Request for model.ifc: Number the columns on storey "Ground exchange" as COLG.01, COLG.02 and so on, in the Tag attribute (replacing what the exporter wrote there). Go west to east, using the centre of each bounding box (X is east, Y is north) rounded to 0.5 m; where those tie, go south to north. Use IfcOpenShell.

First a look at what the model holds.

```python
import ifcopenshell
import ifcopenshell.util.element
import ifcopenshell.util.placement

model = ifcopenshell.open("model.ifc")
print(model.schema)
storey = next(s for s in model.by_type("IfcBuildingStorey") if s.Name == "Ground exchange")
columns = [e for e in ifcopenshell.util.element.get_decomposition(storey) if e.is_a("IfcColumn")]
for e in sorted(columns, key=lambda e: e.id()):
    origin = ifcopenshell.util.placement.get_local_placement(e.ObjectPlacement)[:3, 3]
    print(e.id(), e.Tag, e.Name, origin.round(2) + 0.0, sep=" | ")
```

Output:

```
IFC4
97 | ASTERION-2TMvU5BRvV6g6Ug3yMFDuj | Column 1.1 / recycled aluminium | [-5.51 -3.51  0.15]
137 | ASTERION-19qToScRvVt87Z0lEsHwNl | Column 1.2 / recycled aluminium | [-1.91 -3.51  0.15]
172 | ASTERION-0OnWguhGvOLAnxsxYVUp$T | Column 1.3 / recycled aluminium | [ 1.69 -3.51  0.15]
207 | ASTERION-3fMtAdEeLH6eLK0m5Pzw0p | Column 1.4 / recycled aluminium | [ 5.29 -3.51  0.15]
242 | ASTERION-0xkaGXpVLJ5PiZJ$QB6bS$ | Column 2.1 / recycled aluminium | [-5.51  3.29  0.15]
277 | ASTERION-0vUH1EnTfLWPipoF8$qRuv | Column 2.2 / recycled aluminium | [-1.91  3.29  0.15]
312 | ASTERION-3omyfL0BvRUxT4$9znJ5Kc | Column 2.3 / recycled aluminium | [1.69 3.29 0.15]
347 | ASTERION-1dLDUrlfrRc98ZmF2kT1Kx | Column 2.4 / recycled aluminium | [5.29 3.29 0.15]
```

```python
import ifcopenshell
import ifcopenshell.geom
import ifcopenshell.util.element
import ifcopenshell.util.shape

model = ifcopenshell.open("model.ifc")
settings = ifcopenshell.geom.settings()
settings.set("use-world-coords", True)


def centre(element):
    shape = ifcopenshell.geom.create_shape(settings, element)
    return ifcopenshell.util.shape.get_bbox_centroid(shape.geometry)


storey = next(s for s in model.by_type("IfcBuildingStorey") if s.Name == "Ground exchange")
columns = [e for e in ifcopenshell.util.element.get_decomposition(storey) if e.is_a("IfcColumn")]

# Insertion points can sit at a corner or the storey origin, so sort by the geometry (in metres).
centres = {e: centre(e) for e in columns}
columns.sort(key=lambda e: (round(centres[e][0] / 0.5), centres[e][1]))

for i, e in enumerate(columns, start=1):
    number = f"COLG.{i:02d}"
    e.Tag = number
    print(e.id(), number)

model.write("model_updated.ifc")
```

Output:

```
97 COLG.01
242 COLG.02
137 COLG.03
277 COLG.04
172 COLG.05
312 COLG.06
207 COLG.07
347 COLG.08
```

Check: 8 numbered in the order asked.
